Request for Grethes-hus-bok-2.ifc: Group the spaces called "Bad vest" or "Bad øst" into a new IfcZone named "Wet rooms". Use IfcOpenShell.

First a look at what the model holds.

```python
import ifcopenshell

model = ifcopenshell.open("Grethes-hus-bok-2.ifc")
print(model.schema)
seen = {}
for space in model.by_type("IfcSpace"):
    seen[space.LongName] = seen.get(space.LongName, 0) + 1
for name, count in sorted(seen.items(), key=str):
    print(count, "x", name)
print("zones:", [z.Name for z in model.by_type("IfcZone")][:20])
```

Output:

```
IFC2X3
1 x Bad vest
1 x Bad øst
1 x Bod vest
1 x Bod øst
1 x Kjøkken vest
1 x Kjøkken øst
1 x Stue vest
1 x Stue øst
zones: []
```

```python
import ifcopenshell
import ifcopenshell.api.group
import ifcopenshell.api.root

model = ifcopenshell.open("Grethes-hus-bok-2.ifc")

names = {"Bad vest", "Bad øst"}
spaces = [s for s in model.by_type("IfcSpace") if s.LongName in names]

zone = ifcopenshell.api.root.create_entity(model, ifc_class="IfcZone", name="Wet rooms")
ifcopenshell.api.group.assign_group(model, products=spaces, group=zone)
print(len(spaces), "spaces in", zone.Name)

model.write("Grethes-hus-bok-2_edited.ifc")
```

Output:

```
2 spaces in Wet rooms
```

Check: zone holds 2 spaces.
